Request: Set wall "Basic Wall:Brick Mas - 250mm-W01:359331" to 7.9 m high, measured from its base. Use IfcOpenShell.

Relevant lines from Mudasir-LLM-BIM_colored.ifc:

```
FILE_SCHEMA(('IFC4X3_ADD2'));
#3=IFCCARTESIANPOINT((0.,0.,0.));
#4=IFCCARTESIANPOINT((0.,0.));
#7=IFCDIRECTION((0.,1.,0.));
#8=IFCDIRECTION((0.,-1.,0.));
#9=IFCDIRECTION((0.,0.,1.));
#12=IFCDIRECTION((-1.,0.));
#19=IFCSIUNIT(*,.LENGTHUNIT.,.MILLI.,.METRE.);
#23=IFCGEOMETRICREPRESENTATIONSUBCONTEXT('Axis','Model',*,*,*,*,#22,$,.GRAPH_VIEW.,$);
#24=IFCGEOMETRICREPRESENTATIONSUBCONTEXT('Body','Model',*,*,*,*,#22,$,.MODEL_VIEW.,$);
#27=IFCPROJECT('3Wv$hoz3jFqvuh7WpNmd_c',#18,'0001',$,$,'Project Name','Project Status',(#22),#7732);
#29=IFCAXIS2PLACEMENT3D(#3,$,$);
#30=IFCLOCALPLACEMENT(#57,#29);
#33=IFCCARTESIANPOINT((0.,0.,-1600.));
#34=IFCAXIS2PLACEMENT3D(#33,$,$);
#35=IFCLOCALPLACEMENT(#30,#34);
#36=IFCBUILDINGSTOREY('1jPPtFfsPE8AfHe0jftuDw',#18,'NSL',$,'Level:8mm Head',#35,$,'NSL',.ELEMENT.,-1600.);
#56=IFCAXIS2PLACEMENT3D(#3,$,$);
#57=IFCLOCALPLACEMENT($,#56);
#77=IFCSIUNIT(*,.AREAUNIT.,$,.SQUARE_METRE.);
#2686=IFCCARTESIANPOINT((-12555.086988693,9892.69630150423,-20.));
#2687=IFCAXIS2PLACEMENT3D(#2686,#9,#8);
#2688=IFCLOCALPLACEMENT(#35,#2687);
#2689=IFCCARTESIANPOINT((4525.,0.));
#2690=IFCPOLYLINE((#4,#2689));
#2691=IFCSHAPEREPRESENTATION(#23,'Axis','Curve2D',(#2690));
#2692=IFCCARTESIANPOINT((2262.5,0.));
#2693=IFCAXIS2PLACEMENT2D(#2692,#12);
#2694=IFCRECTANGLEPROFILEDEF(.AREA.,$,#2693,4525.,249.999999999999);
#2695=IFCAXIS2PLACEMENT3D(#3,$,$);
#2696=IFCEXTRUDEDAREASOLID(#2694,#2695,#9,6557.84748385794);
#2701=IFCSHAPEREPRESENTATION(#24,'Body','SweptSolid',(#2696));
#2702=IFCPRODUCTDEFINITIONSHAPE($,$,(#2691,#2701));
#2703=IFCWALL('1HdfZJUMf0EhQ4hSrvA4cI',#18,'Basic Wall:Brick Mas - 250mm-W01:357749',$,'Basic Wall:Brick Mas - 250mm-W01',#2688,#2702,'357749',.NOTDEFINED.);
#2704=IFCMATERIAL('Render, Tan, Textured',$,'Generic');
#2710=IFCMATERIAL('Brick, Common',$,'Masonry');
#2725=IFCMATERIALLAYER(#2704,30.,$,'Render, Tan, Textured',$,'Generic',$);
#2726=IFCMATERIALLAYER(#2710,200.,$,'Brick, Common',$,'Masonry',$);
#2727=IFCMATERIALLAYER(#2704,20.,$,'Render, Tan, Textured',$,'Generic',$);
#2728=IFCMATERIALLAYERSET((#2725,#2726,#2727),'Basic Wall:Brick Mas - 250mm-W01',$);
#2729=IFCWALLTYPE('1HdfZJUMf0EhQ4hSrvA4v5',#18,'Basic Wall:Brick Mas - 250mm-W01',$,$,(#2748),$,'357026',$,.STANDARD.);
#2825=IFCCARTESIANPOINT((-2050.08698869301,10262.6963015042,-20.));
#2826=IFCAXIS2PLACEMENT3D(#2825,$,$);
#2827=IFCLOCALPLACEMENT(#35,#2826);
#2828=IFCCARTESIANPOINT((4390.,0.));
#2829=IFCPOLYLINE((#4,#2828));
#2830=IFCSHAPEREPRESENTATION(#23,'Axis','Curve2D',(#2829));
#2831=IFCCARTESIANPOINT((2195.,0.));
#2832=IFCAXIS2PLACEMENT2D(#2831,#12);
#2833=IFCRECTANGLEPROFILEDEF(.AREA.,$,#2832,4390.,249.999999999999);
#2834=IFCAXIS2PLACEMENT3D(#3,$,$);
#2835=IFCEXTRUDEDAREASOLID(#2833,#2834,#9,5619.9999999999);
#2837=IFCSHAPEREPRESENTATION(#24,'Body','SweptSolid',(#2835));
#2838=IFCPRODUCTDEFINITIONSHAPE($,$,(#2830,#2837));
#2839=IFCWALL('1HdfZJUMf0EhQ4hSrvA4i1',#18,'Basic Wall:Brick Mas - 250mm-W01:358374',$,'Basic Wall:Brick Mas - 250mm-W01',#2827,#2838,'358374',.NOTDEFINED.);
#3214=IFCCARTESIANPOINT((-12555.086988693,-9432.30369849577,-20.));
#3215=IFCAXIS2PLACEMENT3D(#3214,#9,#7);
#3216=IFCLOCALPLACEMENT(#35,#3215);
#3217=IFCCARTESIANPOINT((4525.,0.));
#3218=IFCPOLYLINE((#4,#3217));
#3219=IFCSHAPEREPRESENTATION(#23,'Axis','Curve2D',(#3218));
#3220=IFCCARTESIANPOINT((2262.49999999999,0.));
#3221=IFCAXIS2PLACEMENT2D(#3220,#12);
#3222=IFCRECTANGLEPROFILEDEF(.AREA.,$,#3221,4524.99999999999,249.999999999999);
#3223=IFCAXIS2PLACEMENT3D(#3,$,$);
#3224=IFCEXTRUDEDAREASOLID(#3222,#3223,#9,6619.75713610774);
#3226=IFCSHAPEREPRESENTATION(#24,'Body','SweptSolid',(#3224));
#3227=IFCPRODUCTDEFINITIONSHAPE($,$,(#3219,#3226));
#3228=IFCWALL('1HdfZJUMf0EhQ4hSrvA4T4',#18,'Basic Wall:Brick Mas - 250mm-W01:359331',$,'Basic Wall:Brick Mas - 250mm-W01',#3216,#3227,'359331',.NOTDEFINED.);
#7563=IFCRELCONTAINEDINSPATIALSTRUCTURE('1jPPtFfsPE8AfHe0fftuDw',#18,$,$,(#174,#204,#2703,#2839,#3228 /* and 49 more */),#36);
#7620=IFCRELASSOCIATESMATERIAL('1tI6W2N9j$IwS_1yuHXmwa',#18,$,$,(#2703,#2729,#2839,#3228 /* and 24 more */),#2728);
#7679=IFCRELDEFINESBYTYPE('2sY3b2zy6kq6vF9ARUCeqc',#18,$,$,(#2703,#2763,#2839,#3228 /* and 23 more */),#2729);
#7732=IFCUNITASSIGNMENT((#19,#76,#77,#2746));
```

```python
import ifcopenshell
import ifcopenshell.geom
import ifcopenshell.util.representation
import ifcopenshell.util.shape
import ifcopenshell.util.unit

model = ifcopenshell.open("Mudasir-LLM-BIM_colored.ifc")
unit_scale = ifcopenshell.util.unit.calculate_unit_scale(model)
settings = ifcopenshell.geom.settings()


def volume(element):
    """Net volume in cubic metres, openings subtracted."""
    shape = ifcopenshell.geom.create_shape(settings, element)
    return ifcopenshell.util.shape.get_volume(shape.geometry)


wall = model.by_guid("1HdfZJUMf0EhQ4hSrvA4T4")
before = volume(wall)

body = ifcopenshell.util.representation.get_representation(wall, "Model", "Body")
solid = body.Items[0]
old_height = solid.Depth
solid.Depth = 7.9 / unit_scale
after = volume(wall)

print(f"height {old_height:g} -> {solid.Depth:g}, volume {before:.3f} -> {after:.3f} m3")

model.write("Mudasir-LLM-BIM_colored_rev.ifc")
```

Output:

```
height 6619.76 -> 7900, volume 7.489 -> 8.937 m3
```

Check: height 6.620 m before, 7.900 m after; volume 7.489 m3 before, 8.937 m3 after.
